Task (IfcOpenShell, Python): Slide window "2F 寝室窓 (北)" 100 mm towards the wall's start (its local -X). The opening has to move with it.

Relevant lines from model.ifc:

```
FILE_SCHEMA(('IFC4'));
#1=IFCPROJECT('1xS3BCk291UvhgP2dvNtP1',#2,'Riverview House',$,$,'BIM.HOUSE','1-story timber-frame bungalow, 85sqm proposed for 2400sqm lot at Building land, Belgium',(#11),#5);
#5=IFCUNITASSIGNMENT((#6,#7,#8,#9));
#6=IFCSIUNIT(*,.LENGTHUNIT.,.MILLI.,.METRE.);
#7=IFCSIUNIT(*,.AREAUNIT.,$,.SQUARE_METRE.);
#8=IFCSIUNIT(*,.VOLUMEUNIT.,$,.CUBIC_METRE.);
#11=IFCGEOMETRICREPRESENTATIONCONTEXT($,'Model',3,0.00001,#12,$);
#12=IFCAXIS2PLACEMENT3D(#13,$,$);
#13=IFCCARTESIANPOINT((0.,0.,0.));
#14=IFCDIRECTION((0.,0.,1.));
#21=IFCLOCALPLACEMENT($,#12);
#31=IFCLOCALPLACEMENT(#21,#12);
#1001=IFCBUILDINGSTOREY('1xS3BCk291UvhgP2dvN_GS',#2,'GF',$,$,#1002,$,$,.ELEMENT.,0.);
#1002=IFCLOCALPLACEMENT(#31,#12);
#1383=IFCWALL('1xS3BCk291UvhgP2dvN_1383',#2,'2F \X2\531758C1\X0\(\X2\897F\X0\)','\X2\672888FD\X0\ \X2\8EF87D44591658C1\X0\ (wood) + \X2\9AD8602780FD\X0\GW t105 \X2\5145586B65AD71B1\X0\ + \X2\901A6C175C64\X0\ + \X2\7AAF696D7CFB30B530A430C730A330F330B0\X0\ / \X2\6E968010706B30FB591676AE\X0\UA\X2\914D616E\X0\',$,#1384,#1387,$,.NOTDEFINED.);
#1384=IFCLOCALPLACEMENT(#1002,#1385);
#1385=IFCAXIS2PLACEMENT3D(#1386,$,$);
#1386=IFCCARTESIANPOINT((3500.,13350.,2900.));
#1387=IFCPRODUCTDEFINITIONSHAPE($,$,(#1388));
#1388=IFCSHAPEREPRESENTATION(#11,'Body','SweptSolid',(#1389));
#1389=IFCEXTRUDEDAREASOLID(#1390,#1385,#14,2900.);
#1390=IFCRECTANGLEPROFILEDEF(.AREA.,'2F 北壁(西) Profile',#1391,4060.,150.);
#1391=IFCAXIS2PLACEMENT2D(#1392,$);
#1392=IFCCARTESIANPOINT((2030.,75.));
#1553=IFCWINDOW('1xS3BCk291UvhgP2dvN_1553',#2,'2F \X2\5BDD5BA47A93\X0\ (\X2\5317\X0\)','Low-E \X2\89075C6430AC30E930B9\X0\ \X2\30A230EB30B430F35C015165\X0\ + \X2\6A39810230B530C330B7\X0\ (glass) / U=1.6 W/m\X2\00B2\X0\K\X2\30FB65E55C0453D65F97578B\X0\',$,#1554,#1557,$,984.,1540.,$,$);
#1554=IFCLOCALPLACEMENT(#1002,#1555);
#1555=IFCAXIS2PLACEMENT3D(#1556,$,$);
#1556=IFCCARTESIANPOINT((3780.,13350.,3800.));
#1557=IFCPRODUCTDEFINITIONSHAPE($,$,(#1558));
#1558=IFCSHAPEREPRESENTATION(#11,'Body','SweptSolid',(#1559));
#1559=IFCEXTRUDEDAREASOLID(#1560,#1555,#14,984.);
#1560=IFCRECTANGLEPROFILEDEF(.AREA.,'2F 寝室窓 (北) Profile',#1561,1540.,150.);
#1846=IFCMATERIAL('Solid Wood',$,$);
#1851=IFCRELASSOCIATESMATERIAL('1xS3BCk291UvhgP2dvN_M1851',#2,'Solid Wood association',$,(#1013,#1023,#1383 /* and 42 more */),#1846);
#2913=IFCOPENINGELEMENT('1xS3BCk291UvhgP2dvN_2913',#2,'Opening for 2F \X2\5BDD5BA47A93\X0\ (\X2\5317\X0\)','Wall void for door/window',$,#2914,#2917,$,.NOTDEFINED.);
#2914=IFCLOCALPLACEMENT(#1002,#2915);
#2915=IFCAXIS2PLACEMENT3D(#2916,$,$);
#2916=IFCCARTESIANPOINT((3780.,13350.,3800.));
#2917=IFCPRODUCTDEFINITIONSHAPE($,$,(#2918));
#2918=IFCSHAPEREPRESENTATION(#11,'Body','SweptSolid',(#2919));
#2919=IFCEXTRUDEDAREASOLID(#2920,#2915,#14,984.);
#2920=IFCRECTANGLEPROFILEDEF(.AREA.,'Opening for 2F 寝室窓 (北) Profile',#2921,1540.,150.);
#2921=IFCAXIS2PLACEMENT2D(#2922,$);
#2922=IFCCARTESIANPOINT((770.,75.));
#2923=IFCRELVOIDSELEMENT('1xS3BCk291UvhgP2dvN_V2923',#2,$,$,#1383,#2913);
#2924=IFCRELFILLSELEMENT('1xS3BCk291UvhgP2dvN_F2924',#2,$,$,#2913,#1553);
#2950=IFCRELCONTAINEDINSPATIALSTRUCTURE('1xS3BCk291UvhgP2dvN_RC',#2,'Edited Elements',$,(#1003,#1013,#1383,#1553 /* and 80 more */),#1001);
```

```python
import ifcopenshell
import ifcopenshell.api.geometry
import ifcopenshell.util.placement
import ifcopenshell.util.unit

model = ifcopenshell.open("model.ifc")
unit_scale = ifcopenshell.util.unit.calculate_unit_scale(model)

window = model.by_guid("1xS3BCk291UvhgP2dvN_1553")
opening = window.FillsVoids[0].RelatingOpeningElement
wall = opening.VoidsElements[0].RelatingBuildingElement

wall_matrix = ifcopenshell.util.placement.get_local_placement(wall.ObjectPlacement)
shift = wall_matrix[:3, 0] * -0.1 / unit_scale
before = ifcopenshell.util.placement.get_local_placement(window.ObjectPlacement)[:3, 3].copy()

# The window is not placed relative to its opening, so move both.
for product in (opening, window):
    matrix = ifcopenshell.util.placement.get_local_placement(product.ObjectPlacement)
    matrix[:3, 3] += shift
    ifcopenshell.api.geometry.edit_object_placement(model, product=product, matrix=matrix, is_si=False)

after = ifcopenshell.util.placement.get_local_placement(window.ObjectPlacement)[:3, 3]
print("window moved by", (after - before).round(3) + 0.0)

model.write("model-out.ifc")
```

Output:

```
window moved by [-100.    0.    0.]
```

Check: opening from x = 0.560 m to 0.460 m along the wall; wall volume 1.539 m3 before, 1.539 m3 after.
